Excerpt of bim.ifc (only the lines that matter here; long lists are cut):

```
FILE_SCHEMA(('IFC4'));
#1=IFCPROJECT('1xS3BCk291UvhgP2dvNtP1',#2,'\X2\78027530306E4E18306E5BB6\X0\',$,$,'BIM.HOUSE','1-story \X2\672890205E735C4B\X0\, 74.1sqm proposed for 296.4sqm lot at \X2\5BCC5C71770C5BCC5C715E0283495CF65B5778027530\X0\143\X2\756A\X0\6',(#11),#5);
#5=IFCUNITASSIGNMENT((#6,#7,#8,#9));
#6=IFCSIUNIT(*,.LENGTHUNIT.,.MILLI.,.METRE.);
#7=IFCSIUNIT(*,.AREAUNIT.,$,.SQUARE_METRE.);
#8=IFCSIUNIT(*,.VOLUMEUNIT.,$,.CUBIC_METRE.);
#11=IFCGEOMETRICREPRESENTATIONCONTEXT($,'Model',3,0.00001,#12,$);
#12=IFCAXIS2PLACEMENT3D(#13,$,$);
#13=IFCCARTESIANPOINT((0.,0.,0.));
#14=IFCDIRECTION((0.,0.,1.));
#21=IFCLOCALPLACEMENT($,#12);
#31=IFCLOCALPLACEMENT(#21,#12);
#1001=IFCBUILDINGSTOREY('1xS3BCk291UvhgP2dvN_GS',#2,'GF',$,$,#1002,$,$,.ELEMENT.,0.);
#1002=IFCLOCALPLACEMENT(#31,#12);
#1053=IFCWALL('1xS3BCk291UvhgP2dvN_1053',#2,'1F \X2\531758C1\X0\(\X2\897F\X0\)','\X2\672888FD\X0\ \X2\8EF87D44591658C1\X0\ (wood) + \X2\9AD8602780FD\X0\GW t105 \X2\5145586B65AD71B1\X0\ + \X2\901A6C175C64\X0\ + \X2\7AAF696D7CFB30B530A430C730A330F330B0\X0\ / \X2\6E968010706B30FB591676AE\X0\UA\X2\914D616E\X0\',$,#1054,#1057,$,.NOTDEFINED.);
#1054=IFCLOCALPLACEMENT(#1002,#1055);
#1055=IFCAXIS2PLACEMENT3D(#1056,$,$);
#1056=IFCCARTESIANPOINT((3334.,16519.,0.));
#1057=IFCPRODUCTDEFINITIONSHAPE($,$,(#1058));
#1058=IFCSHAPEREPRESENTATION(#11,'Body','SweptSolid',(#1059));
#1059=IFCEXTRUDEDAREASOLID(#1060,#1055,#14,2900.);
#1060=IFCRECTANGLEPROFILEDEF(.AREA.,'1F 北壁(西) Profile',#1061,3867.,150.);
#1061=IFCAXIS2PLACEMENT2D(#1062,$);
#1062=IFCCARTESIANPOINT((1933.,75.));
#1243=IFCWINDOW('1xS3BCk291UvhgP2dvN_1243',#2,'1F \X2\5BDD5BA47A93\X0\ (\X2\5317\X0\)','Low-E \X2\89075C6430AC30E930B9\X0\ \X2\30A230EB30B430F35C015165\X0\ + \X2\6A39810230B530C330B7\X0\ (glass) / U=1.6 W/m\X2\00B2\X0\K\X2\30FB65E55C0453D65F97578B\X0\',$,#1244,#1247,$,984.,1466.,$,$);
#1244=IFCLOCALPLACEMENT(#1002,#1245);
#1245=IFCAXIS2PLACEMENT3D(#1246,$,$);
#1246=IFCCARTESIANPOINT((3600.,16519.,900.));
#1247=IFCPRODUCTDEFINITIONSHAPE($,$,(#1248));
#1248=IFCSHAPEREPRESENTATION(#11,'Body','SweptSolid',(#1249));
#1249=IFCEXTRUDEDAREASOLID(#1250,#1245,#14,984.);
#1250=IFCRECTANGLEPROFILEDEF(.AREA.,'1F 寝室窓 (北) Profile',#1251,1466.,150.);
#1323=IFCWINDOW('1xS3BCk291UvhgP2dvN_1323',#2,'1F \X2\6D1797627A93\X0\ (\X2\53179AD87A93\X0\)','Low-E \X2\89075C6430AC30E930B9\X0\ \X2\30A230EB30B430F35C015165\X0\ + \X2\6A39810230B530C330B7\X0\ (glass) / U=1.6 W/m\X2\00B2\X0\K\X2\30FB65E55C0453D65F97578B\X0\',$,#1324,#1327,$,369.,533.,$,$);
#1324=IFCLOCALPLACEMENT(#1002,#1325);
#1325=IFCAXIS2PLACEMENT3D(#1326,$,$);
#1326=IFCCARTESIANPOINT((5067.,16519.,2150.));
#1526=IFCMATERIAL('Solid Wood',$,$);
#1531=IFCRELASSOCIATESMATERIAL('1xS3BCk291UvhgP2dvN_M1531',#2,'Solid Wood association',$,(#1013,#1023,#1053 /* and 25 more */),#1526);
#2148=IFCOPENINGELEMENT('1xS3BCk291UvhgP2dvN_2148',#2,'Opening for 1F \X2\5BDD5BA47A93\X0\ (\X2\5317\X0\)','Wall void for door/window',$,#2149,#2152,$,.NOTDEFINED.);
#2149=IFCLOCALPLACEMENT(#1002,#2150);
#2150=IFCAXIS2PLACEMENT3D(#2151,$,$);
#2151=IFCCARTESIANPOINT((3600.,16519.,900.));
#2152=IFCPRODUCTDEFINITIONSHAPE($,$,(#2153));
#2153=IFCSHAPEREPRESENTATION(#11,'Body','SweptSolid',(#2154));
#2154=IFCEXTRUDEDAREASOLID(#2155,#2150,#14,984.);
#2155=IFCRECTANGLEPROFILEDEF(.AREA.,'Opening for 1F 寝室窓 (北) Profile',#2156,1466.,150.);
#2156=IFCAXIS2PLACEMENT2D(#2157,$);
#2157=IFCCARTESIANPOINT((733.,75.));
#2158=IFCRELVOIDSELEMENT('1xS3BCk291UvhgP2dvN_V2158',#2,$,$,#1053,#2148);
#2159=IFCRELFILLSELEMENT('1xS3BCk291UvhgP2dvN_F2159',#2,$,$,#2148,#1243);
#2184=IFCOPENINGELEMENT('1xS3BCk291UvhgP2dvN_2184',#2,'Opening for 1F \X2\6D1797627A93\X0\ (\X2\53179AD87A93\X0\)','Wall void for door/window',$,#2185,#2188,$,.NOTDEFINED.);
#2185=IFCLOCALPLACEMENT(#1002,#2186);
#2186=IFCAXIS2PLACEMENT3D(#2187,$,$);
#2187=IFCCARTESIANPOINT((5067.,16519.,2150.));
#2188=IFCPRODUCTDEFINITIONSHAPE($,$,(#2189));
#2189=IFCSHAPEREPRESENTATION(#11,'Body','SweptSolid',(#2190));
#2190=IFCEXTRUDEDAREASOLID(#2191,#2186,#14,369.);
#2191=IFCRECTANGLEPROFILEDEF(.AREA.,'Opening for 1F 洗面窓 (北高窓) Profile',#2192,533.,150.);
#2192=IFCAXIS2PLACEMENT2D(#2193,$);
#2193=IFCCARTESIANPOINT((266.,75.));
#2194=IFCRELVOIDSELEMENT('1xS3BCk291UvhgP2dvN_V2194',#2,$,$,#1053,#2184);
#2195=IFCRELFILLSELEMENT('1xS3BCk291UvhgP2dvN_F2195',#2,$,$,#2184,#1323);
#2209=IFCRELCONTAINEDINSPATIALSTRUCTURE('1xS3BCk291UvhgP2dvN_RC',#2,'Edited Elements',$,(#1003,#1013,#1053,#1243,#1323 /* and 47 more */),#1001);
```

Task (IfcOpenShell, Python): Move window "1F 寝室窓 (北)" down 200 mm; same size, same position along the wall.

```python
import numpy as np
import ifcopenshell
import ifcopenshell.api.geometry
import ifcopenshell.util.placement
import ifcopenshell.util.unit

model = ifcopenshell.open("bim.ifc")
unit_scale = ifcopenshell.util.unit.calculate_unit_scale(model)

window = model.by_guid("1xS3BCk291UvhgP2dvN_1243")
opening = window.FillsVoids[0].RelatingOpeningElement
dz = -0.2 / unit_scale

shift = np.array([0.0, 0.0, dz])
# The window is not placed relative to its opening, so move both.
for product in (opening, window):
    matrix = ifcopenshell.util.placement.get_local_placement(product.ObjectPlacement)
    matrix[:3, 3] += shift
    ifcopenshell.api.geometry.edit_object_placement(model, product=product, matrix=matrix, is_si=False)

print(f"moved by {dz * unit_scale:+.3f} m")

model.write("bim_edited.ifc")
```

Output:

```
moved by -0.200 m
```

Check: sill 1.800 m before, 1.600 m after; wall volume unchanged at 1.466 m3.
